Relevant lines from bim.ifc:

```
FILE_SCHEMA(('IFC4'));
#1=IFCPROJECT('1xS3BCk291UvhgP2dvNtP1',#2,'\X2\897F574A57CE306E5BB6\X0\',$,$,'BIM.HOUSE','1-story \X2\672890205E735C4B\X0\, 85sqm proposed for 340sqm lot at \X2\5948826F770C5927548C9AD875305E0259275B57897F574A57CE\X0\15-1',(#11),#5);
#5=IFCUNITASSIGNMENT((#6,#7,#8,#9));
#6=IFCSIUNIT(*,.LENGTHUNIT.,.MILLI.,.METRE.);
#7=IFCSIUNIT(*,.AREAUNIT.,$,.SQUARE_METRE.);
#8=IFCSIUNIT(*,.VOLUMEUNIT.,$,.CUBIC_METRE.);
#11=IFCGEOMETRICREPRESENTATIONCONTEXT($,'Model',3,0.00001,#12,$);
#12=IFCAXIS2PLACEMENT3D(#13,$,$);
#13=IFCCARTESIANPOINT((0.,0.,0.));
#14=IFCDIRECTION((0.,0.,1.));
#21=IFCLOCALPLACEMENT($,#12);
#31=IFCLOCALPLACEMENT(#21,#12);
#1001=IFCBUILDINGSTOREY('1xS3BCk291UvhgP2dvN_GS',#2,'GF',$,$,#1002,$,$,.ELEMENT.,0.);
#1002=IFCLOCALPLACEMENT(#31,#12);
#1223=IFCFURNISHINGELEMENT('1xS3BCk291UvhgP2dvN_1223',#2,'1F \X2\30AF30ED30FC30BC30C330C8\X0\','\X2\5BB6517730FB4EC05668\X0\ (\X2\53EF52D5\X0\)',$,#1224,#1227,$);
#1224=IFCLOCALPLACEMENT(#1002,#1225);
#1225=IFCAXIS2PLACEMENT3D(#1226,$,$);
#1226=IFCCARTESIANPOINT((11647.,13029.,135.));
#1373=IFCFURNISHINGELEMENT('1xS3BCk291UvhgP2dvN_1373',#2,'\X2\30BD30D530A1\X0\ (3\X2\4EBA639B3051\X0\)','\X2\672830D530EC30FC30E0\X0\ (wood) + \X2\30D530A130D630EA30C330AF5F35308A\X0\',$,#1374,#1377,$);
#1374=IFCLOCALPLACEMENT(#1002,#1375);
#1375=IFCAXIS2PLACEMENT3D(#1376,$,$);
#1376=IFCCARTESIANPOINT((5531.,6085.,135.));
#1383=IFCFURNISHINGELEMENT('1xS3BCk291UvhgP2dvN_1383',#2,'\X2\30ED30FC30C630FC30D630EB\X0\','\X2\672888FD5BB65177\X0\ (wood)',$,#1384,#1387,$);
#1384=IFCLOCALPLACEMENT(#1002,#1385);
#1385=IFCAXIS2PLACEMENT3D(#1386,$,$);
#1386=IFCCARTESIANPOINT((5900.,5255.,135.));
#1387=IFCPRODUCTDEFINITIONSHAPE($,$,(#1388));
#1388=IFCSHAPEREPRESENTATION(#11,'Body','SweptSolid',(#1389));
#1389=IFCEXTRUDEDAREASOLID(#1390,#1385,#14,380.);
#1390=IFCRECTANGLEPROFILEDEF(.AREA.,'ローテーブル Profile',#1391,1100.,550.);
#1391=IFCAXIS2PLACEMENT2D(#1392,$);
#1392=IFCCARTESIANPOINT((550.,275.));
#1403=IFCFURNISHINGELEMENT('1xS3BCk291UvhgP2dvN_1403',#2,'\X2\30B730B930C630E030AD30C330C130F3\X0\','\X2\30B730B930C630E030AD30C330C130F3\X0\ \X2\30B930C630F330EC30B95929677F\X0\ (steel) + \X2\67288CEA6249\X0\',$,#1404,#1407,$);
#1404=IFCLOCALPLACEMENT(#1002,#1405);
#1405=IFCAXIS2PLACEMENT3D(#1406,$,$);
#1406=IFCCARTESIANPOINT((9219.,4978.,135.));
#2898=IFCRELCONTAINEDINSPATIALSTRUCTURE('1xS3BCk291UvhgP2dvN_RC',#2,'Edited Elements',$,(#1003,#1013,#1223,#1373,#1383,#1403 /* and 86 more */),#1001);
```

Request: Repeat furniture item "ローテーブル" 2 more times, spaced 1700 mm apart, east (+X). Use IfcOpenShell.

```python
import numpy as np
import ifcopenshell
import ifcopenshell.api.geometry
import ifcopenshell.api.root
import ifcopenshell.util.element
import ifcopenshell.util.placement
import ifcopenshell.util.unit

model = ifcopenshell.open("bim.ifc")
unit_scale = ifcopenshell.util.unit.calculate_unit_scale(model)


def reuse_history(source, copy):
    """copy_class also copies each property set's owner history, people and application; keep the originals."""
    for rel in copy.IsDefinedBy:
        if rel.is_a("IfcRelDefinesByProperties") and (history := rel.RelatingPropertyDefinition.OwnerHistory):
            rel.RelatingPropertyDefinition.OwnerHistory = source.OwnerHistory
            ifcopenshell.util.element.remove_deep2(model, history)


source = model.by_guid("1xS3BCk291UvhgP2dvN_1383")
base = ifcopenshell.util.placement.get_local_placement(source.ObjectPlacement)
step = np.array([1.0, 0.0, 0.0]) * 1.7 / unit_scale

for i in range(1, 3):
    copy = ifcopenshell.api.root.copy_class(model, product=source)
    copy.Representation = ifcopenshell.util.element.copy_deep(
        model, source.Representation, exclude=["IfcGeometricRepresentationContext", "IfcRepresentationMap"]
    )
    reuse_history(source, copy)
    matrix = base.copy()
    matrix[:3, 3] += i * step
    print("added at", matrix[:3, 3].round(3) + 0.0)
    ifcopenshell.api.geometry.edit_object_placement(model, product=copy, matrix=matrix, is_si=False)

model.write("bim_updated.ifc")
```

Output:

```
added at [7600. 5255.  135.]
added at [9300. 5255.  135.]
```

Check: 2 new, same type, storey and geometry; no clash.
